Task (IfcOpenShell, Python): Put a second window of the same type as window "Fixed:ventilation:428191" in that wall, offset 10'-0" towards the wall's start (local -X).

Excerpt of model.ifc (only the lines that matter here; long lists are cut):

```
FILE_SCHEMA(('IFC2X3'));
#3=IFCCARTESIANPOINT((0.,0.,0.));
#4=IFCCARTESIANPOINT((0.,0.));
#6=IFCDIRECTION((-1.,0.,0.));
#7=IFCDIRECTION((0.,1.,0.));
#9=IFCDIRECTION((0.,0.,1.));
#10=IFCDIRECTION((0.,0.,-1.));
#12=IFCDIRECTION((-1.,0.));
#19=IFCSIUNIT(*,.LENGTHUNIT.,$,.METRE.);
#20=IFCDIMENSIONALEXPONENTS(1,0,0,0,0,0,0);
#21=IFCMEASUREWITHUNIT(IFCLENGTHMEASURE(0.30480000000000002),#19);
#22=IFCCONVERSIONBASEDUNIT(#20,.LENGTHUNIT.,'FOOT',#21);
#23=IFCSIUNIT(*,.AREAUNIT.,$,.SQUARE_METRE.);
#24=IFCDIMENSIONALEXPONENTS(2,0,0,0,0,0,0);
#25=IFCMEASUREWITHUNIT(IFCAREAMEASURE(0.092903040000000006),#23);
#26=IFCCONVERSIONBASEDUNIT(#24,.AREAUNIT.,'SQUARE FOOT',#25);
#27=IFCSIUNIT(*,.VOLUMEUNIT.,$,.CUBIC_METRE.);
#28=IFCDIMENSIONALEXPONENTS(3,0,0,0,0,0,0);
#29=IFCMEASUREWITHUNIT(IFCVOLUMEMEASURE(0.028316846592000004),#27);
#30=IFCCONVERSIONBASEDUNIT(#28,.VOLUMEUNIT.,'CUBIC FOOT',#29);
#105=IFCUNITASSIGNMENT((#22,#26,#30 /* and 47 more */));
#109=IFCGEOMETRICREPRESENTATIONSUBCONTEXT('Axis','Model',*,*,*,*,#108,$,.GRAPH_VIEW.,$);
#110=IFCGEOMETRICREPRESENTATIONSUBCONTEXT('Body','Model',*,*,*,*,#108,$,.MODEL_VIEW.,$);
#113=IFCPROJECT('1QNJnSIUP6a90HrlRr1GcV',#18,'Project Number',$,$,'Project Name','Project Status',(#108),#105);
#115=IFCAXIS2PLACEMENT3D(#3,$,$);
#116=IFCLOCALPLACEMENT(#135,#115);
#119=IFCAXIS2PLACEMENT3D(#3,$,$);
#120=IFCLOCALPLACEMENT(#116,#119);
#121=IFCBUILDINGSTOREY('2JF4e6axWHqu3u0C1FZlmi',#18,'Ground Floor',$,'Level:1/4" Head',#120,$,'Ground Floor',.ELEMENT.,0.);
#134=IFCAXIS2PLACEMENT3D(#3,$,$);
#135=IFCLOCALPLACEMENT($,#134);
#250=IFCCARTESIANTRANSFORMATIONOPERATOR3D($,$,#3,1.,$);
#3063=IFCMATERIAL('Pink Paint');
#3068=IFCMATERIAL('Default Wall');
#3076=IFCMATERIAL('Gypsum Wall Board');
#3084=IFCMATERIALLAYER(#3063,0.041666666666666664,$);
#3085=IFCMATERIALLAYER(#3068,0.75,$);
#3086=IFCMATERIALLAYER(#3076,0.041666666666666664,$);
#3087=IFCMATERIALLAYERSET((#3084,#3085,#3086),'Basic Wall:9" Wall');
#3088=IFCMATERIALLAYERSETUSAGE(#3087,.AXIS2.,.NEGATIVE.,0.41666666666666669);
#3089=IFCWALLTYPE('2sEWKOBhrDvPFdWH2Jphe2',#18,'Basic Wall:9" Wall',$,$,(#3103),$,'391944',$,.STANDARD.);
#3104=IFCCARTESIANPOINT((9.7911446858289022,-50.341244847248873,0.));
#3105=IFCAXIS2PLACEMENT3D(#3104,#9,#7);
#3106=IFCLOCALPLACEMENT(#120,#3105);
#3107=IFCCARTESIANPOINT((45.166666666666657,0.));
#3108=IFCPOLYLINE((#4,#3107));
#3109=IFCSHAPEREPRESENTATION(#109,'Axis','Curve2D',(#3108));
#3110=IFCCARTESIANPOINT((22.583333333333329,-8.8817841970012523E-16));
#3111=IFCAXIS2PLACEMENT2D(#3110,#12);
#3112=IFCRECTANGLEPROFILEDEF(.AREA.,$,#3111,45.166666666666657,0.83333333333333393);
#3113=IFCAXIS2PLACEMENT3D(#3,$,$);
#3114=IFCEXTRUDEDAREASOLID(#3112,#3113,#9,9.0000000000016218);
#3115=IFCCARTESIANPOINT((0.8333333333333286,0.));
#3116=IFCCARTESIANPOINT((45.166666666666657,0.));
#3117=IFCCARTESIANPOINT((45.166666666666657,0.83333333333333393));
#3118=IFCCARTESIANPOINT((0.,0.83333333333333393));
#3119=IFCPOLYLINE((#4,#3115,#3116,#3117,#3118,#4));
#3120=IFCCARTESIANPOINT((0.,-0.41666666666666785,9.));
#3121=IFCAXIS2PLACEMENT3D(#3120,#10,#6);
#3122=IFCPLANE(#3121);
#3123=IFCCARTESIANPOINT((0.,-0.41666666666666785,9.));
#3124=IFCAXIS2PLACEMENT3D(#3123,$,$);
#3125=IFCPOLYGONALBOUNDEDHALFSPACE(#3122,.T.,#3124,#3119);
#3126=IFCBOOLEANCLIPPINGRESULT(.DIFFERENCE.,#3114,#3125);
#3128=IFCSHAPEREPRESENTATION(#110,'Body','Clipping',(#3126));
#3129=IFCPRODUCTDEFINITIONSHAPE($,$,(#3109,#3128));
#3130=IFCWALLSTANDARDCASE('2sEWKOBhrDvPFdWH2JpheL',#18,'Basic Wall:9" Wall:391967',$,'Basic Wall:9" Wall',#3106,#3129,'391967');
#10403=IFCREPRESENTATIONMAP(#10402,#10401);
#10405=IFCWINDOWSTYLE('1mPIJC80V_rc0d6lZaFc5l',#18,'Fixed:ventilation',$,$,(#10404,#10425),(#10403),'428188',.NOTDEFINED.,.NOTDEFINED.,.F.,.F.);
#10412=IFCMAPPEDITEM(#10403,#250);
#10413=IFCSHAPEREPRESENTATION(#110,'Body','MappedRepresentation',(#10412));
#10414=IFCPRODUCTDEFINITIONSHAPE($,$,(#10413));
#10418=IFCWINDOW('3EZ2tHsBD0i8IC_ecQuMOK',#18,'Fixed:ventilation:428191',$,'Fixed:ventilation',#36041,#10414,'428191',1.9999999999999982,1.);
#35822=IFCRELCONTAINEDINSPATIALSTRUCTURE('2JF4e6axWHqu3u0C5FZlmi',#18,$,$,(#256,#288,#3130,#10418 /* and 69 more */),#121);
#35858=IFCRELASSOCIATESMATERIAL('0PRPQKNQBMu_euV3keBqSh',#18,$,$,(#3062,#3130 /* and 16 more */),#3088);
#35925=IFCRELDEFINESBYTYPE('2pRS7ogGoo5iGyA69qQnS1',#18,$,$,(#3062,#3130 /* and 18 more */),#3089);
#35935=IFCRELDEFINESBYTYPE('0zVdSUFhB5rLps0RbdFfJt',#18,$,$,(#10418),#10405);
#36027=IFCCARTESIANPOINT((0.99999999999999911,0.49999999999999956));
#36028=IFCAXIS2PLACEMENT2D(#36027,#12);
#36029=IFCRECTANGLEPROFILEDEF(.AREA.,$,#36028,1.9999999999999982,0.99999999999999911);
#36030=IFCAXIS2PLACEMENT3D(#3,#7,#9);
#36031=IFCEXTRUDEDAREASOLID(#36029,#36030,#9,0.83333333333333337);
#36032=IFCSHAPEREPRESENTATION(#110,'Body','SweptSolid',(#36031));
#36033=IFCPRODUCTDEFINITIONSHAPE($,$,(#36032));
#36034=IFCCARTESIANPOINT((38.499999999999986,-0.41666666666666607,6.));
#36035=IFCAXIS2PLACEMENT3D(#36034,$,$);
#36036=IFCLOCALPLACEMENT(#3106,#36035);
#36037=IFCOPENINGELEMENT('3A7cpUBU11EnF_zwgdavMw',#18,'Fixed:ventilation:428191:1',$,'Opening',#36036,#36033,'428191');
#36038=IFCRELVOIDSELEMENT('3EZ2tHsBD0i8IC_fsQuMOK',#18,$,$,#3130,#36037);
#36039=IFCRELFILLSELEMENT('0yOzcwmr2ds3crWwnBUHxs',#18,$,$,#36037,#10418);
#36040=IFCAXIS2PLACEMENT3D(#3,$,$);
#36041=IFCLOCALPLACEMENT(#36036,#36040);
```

```python
import ifcopenshell
import ifcopenshell.api.feature
import ifcopenshell.api.geometry
import ifcopenshell.api.root
import ifcopenshell.geom
import ifcopenshell.util.element
import ifcopenshell.util.placement
import ifcopenshell.util.shape
import ifcopenshell.util.unit

model = ifcopenshell.open("model.ifc")
unit_scale = ifcopenshell.util.unit.calculate_unit_scale(model)
settings = ifcopenshell.geom.settings()


def volume(element):
    """Net volume in cubic metres, openings subtracted."""
    shape = ifcopenshell.geom.create_shape(settings, element)
    return ifcopenshell.util.shape.get_volume(shape.geometry)


def reuse_history(source, copy):
    """copy_class also copies each property set's owner history, people and application; keep the originals."""
    for rel in copy.IsDefinedBy:
        if rel.is_a("IfcRelDefinesByProperties") and (history := rel.RelatingPropertyDefinition.OwnerHistory):
            rel.RelatingPropertyDefinition.OwnerHistory = source.OwnerHistory
            ifcopenshell.util.element.remove_deep2(model, history)


window = model.by_id(10418)
opening = window.FillsVoids[0].RelatingOpeningElement
wall = opening.VoidsElements[0].RelatingBuildingElement
before = volume(wall)
shift = ifcopenshell.util.placement.get_local_placement(wall.ObjectPlacement)[:3, 0] * -120 * 0.0254 / unit_scale

# copy_class copies the void relationship, type, container and properties, but no geometry.
new_opening = ifcopenshell.api.root.copy_class(model, product=opening)
new_opening.Representation = ifcopenshell.util.element.copy_deep(
    model, opening.Representation, exclude=["IfcGeometricRepresentationContext", "IfcRepresentationMap"]
)
new_opening.Name = "Fixed:ventilation"
new_opening.Tag = None
new_window = ifcopenshell.api.root.copy_class(model, product=window)
new_window.Representation = ifcopenshell.util.element.copy_deep(
    model, window.Representation, exclude=["IfcGeometricRepresentationContext", "IfcRepresentationMap"]
)
new_window.Name = "Fixed:ventilation"
new_window.Tag = None
reuse_history(window, new_window)
fills = ifcopenshell.api.feature.add_filling(model, opening=new_opening, element=new_window)
fills.OwnerHistory = new_window.OwnerHistory  # required in IFC2X3

for old, new in ((opening, new_opening), (window, new_window)):
    matrix = ifcopenshell.util.placement.get_local_placement(old.ObjectPlacement)
    matrix[:3, 3] += shift
    ifcopenshell.api.geometry.edit_object_placement(model, product=new, matrix=matrix, is_si=False)

after = volume(wall)

print(f"wall volume {before:.3f} -> {after:.3f} m3")

model.write("model_updated.ifc")
```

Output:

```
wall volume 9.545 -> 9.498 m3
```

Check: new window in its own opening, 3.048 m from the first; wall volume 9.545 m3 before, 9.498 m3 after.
